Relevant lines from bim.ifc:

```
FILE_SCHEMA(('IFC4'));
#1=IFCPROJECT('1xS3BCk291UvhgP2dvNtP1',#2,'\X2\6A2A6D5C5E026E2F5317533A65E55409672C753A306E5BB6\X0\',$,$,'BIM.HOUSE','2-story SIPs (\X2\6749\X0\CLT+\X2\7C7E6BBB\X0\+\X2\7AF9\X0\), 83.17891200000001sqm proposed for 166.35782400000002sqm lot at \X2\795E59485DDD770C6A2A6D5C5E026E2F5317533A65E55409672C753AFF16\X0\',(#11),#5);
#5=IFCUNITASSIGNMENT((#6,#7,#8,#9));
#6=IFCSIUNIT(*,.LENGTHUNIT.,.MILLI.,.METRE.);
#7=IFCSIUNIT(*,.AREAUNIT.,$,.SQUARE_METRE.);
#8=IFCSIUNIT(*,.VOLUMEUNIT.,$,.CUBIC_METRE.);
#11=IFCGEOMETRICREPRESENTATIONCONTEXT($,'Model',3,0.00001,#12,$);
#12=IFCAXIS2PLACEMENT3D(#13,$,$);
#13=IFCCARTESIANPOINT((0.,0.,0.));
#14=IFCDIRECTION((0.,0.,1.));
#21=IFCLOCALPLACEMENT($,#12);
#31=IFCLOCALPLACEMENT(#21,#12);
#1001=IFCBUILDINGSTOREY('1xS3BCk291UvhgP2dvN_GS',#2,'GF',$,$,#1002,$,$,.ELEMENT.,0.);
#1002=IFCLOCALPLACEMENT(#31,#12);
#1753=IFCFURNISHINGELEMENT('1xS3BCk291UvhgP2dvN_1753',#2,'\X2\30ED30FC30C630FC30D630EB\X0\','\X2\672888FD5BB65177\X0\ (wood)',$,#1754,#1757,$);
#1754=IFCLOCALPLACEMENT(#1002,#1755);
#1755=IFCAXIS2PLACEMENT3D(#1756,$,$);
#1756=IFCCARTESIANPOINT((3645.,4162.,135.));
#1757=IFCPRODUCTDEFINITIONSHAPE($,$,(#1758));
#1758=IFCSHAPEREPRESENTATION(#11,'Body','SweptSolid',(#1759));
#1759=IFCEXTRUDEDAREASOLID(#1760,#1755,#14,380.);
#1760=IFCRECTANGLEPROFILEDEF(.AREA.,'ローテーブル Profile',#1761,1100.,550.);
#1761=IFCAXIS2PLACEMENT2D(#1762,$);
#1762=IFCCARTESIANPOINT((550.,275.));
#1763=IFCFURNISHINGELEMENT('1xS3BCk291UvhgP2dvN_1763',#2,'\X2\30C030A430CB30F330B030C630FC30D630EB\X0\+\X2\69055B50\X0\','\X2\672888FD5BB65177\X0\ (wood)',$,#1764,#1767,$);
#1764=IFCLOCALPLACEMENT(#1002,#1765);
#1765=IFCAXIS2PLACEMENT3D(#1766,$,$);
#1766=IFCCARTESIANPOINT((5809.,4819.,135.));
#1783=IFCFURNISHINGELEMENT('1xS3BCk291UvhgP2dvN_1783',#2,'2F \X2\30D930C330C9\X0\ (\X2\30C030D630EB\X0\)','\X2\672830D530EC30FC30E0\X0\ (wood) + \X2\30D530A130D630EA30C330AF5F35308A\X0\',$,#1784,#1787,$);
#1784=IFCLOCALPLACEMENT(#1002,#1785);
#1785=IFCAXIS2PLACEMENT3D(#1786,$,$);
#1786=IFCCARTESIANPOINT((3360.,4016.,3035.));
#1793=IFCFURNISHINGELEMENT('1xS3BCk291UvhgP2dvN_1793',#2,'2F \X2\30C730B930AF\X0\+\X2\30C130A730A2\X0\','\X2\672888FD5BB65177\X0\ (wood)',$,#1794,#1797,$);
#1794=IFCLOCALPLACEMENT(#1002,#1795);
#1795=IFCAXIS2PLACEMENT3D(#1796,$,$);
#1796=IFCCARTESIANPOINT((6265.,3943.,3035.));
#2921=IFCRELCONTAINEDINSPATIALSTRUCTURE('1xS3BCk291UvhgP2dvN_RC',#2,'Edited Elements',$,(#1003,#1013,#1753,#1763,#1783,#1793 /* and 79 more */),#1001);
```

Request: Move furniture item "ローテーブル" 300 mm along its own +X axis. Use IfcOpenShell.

```python
import ifcopenshell
import ifcopenshell.api.geometry
import ifcopenshell.util.placement
import ifcopenshell.util.unit

model = ifcopenshell.open("bim.ifc")
unit_scale = ifcopenshell.util.unit.calculate_unit_scale(model)

item = model.by_guid("1xS3BCk291UvhgP2dvN_1753")
matrix = ifcopenshell.util.placement.get_local_placement(item.ObjectPlacement)
matrix[:3, 3] += matrix[:3, 0] * 0.3 / unit_scale
ifcopenshell.api.geometry.edit_object_placement(model, product=item, matrix=matrix, is_si=False)

print(ifcopenshell.util.placement.get_local_placement(item.ObjectPlacement).round(3) + 0.0)

model.write("bim_updated.ifc")
```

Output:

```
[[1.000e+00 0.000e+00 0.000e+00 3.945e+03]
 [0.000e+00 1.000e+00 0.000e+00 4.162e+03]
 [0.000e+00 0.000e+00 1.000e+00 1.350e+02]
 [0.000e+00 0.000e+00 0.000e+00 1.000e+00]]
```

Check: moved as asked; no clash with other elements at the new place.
